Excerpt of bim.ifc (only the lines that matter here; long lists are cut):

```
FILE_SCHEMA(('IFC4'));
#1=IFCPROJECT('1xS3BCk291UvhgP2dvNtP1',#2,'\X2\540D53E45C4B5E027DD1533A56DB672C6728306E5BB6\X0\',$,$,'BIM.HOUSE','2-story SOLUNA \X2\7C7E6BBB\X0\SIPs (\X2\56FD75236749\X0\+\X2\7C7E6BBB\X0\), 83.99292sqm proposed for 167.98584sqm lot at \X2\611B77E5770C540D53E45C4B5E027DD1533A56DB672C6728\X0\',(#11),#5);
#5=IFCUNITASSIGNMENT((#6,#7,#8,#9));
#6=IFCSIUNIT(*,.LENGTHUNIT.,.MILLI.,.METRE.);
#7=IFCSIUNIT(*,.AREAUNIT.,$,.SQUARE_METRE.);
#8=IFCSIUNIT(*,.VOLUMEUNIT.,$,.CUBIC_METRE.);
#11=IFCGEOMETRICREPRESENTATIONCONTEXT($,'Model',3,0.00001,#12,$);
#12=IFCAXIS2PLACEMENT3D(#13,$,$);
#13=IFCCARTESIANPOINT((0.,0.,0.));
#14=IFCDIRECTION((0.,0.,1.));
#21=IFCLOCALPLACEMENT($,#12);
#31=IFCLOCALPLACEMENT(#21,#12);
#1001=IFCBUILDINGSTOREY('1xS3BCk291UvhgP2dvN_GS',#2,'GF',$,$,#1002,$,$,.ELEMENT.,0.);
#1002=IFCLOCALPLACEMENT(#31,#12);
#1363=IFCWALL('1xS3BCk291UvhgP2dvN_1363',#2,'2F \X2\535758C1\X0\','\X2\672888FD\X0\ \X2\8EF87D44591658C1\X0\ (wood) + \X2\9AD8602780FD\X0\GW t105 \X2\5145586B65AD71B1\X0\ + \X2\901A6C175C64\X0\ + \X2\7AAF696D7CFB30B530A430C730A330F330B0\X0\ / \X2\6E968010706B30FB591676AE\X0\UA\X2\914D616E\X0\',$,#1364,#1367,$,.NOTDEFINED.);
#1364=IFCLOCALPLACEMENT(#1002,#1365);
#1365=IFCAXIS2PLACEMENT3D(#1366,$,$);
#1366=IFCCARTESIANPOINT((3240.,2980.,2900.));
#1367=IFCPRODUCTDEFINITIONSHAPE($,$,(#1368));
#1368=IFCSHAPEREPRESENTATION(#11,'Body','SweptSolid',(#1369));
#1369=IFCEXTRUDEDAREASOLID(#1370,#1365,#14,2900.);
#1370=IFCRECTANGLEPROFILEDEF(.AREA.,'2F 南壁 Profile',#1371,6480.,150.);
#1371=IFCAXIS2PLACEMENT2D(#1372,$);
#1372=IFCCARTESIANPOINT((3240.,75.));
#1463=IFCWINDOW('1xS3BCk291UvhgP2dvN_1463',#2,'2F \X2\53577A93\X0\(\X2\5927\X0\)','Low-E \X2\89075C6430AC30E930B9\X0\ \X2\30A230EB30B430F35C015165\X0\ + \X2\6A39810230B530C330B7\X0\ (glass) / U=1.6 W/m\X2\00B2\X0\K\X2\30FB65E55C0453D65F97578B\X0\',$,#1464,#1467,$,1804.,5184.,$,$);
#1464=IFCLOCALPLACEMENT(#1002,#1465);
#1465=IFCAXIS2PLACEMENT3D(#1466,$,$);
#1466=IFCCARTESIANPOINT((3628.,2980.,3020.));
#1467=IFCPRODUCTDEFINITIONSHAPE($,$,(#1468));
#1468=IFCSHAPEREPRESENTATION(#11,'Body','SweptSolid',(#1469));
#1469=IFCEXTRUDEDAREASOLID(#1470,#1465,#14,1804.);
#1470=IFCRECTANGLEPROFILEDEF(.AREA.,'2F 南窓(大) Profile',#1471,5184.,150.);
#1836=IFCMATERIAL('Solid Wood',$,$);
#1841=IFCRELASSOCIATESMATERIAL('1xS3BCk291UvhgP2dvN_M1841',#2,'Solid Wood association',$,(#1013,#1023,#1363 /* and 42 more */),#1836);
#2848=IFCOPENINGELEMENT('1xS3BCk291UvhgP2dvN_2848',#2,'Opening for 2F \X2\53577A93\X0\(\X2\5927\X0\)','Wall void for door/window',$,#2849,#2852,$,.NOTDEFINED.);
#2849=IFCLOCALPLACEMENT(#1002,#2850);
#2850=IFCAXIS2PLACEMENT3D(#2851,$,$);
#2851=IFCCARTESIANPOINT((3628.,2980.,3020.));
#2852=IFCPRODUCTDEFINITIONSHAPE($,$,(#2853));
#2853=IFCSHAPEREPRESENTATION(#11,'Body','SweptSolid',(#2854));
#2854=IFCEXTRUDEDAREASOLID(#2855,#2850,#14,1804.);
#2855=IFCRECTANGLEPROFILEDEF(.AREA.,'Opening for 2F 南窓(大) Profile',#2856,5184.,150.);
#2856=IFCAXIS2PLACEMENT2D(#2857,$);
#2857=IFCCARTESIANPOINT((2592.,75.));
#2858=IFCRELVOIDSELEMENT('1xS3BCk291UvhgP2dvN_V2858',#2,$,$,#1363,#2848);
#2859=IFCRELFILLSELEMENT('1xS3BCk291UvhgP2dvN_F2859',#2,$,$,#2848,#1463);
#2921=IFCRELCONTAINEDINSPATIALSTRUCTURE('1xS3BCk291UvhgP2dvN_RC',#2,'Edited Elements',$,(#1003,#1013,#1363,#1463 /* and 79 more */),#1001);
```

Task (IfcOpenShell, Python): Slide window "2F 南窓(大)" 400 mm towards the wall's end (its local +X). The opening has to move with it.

```python
import ifcopenshell
import ifcopenshell.api.geometry
import ifcopenshell.util.placement

model = ifcopenshell.open("bim.ifc")

window = model.by_guid("1xS3BCk291UvhgP2dvN_1463")
opening = window.FillsVoids[0].RelatingOpeningElement
wall = opening.VoidsElements[0].RelatingBuildingElement

wall_matrix = ifcopenshell.util.placement.get_local_placement(wall.ObjectPlacement)
shift = wall_matrix[:3, 0] * 400.0
before = ifcopenshell.util.placement.get_local_placement(window.ObjectPlacement)[:3, 3].copy()

# The window is not placed relative to its opening, so move both.
for product in (opening, window):
    matrix = ifcopenshell.util.placement.get_local_placement(product.ObjectPlacement)
    matrix[:3, 3] += shift
    ifcopenshell.api.geometry.edit_object_placement(model, product=product, matrix=matrix, is_si=False)

after = ifcopenshell.util.placement.get_local_placement(window.ObjectPlacement)[:3, 3]
print("window moved by", (after - before).round(3) + 0.0)

model.write("bim-out.ifc")
```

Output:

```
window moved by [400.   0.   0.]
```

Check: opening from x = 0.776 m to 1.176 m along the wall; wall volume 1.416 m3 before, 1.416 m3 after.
